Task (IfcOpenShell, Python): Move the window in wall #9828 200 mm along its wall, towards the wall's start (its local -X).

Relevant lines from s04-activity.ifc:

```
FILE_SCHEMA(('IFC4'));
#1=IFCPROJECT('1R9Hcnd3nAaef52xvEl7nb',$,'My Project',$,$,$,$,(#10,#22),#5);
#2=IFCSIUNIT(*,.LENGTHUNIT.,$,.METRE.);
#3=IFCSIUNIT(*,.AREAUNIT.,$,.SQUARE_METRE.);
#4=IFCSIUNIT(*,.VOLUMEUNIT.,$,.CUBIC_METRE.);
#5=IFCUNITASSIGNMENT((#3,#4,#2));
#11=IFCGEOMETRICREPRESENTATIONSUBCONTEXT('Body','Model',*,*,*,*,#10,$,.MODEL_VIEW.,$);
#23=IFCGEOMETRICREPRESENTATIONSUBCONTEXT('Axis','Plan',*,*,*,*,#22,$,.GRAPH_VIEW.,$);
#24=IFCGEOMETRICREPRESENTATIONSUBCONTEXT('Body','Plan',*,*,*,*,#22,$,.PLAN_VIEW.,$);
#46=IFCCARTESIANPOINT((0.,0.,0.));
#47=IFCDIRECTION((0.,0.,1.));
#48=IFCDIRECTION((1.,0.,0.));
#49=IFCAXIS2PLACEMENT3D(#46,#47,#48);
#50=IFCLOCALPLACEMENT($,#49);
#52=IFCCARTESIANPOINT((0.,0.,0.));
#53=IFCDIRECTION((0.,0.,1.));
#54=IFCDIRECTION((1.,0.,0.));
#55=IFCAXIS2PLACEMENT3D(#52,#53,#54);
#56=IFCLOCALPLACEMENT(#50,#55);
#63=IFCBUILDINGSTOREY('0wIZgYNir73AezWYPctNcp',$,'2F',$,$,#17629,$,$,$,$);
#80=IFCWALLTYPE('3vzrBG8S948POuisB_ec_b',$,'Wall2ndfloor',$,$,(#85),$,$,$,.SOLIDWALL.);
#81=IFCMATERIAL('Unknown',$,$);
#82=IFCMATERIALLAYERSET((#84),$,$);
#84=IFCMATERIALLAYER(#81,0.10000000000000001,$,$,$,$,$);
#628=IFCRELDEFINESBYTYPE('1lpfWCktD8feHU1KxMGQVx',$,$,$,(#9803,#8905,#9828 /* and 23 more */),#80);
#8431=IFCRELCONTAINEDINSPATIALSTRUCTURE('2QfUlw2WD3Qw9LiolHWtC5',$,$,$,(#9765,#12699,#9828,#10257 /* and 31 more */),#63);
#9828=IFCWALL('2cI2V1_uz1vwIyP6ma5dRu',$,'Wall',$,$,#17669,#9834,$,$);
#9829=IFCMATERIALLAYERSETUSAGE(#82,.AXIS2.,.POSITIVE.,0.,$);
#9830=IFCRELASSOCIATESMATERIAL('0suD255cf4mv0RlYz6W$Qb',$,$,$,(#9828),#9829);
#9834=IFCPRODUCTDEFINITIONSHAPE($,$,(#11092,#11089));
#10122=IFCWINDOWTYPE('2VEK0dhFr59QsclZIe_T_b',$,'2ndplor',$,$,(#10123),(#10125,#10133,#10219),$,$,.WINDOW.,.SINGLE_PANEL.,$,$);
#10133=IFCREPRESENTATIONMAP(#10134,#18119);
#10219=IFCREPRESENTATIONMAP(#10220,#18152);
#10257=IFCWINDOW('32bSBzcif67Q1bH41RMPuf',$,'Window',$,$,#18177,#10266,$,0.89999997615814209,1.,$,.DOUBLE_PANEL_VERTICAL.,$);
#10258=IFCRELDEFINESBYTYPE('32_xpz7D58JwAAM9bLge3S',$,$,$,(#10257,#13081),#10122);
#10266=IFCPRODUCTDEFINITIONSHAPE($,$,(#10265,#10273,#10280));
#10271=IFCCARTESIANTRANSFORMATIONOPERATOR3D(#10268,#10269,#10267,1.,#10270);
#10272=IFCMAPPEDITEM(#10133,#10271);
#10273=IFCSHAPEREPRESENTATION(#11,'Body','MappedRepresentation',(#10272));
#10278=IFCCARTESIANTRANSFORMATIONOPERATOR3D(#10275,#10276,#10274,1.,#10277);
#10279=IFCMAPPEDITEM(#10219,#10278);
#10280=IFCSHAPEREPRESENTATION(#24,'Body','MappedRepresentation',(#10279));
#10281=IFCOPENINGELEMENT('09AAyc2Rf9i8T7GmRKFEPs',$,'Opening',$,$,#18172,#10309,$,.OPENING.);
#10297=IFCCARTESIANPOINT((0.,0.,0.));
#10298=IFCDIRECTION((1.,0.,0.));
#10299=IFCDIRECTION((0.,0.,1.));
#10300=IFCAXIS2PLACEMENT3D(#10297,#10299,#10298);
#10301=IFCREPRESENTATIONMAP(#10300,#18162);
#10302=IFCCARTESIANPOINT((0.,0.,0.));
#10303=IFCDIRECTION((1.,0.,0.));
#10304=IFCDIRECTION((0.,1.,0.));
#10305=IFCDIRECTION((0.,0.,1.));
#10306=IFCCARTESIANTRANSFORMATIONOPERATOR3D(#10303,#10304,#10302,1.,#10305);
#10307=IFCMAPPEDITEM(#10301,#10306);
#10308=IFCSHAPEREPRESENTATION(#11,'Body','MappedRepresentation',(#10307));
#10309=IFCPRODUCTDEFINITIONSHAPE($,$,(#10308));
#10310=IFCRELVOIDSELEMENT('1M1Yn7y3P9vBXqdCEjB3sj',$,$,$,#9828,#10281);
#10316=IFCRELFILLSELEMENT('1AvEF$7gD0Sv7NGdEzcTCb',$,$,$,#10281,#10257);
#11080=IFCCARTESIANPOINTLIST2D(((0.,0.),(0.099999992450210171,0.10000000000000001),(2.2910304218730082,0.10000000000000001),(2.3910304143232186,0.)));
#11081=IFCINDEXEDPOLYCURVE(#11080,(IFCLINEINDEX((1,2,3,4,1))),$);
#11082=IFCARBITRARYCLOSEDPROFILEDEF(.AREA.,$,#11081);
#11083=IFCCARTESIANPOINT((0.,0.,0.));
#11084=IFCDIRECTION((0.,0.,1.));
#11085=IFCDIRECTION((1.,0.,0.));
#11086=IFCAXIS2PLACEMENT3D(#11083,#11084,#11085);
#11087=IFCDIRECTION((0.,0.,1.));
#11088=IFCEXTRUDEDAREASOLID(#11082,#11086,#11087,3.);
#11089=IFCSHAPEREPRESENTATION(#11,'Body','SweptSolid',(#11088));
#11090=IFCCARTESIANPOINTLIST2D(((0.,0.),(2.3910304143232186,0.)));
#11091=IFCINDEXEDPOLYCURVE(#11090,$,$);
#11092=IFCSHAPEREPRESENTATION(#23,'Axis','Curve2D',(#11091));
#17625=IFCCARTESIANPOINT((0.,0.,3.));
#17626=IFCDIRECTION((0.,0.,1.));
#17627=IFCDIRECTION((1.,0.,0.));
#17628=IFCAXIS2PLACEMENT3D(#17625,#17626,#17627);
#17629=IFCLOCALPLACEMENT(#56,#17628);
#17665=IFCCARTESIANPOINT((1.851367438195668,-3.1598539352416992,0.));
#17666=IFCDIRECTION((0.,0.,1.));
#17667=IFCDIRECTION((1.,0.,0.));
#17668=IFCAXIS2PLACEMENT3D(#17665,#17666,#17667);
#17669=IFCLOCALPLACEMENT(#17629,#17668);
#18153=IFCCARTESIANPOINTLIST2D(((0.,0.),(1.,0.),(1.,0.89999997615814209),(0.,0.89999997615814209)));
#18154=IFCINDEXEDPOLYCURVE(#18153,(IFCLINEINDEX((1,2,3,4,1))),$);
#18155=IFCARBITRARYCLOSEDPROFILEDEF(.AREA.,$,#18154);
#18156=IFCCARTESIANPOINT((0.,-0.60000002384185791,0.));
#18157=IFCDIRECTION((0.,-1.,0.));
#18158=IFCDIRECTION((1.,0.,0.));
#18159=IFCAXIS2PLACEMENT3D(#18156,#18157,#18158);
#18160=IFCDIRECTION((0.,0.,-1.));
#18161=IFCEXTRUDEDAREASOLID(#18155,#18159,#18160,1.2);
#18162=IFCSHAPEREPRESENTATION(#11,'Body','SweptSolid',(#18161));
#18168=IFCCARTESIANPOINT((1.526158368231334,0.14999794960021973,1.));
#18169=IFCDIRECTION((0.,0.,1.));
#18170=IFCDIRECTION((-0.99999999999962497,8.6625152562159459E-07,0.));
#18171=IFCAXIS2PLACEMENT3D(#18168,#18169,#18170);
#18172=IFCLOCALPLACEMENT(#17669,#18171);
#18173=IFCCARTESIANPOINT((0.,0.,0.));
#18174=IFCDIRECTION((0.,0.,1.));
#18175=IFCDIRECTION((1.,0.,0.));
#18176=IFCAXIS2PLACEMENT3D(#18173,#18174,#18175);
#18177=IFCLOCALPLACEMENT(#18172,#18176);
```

```python
import ifcopenshell
import ifcopenshell.api.geometry
import ifcopenshell.util.placement
import ifcopenshell.util.unit

model = ifcopenshell.open("s04-activity.ifc")
unit_scale = ifcopenshell.util.unit.calculate_unit_scale(model)

window = model.by_guid("32bSBzcif67Q1bH41RMPuf")
opening = window.FillsVoids[0].RelatingOpeningElement
wall = opening.VoidsElements[0].RelatingBuildingElement

wall_matrix = ifcopenshell.util.placement.get_local_placement(wall.ObjectPlacement)
shift = wall_matrix[:3, 0] * -0.2 / unit_scale
before = ifcopenshell.util.placement.get_local_placement(window.ObjectPlacement)[:3, 3].copy()

# The window is placed relative to its opening, so it follows when the opening moves.
matrix = ifcopenshell.util.placement.get_local_placement(opening.ObjectPlacement)
matrix[:3, 3] += shift
ifcopenshell.api.geometry.edit_object_placement(
    model, product=opening, matrix=matrix, is_si=False, should_transform_children=True
)

after = ifcopenshell.util.placement.get_local_placement(window.ObjectPlacement)[:3, 3]
print("window moved by", (after - before).round(3) + 0.0)

model.write("s04-activity_v2.ifc")
```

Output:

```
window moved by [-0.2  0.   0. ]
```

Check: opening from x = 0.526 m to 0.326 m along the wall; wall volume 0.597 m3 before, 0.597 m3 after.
